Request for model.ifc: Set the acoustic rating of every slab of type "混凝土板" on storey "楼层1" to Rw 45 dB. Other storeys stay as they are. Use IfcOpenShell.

First a look at what the model holds.

```python
import ifcopenshell
import ifcopenshell.util.element

model = ifcopenshell.open("model.ifc")
print(model.schema)
storey = next(s for s in model.by_type("IfcBuildingStorey") if s.Name == "楼层1")
slabs = [e for e in ifcopenshell.util.element.get_decomposition(storey) if e.is_a("IfcSlab")]
seen = {}
for e in slabs:
    element_type = ifcopenshell.util.element.get_type(e)
    key = (element_type.Name if element_type != e and element_type else None, ifcopenshell.util.element.get_pset(e, "Pset_SlabCommon", "AcousticRating"))
    seen[key] = seen.get(key, 0) + 1
for (name, value), count in sorted(seen.items(), key=str):
    print(count, "x", name, "|", value)
```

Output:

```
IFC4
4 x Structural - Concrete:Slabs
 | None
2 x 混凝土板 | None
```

```python
import ifcopenshell
import ifcopenshell.api.pset
import ifcopenshell.util.element

model = ifcopenshell.open("model.ifc")

storey = next(s for s in model.by_type("IfcBuildingStorey") if s.Name == "楼层1")
slabs = [e for e in ifcopenshell.util.element.get_decomposition(storey) if e.is_a("IfcSlab")]

count = 0
for e in slabs:
    element_type = ifcopenshell.util.element.get_type(e)
    if element_type in (None, e) or element_type.Name != "混凝土板":
        continue
    # add_pset returns the element's existing set when there is one.
    pset = ifcopenshell.api.pset.add_pset(model, product=e, name="Pset_SlabCommon")
    ifcopenshell.api.pset.edit_pset(model, pset=pset, properties={"AcousticRating": "Rw 45 dB"})
    count += 1

print(count, "slabs updated")

model.write("model_rev.ifc")
```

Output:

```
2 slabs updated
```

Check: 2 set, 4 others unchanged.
